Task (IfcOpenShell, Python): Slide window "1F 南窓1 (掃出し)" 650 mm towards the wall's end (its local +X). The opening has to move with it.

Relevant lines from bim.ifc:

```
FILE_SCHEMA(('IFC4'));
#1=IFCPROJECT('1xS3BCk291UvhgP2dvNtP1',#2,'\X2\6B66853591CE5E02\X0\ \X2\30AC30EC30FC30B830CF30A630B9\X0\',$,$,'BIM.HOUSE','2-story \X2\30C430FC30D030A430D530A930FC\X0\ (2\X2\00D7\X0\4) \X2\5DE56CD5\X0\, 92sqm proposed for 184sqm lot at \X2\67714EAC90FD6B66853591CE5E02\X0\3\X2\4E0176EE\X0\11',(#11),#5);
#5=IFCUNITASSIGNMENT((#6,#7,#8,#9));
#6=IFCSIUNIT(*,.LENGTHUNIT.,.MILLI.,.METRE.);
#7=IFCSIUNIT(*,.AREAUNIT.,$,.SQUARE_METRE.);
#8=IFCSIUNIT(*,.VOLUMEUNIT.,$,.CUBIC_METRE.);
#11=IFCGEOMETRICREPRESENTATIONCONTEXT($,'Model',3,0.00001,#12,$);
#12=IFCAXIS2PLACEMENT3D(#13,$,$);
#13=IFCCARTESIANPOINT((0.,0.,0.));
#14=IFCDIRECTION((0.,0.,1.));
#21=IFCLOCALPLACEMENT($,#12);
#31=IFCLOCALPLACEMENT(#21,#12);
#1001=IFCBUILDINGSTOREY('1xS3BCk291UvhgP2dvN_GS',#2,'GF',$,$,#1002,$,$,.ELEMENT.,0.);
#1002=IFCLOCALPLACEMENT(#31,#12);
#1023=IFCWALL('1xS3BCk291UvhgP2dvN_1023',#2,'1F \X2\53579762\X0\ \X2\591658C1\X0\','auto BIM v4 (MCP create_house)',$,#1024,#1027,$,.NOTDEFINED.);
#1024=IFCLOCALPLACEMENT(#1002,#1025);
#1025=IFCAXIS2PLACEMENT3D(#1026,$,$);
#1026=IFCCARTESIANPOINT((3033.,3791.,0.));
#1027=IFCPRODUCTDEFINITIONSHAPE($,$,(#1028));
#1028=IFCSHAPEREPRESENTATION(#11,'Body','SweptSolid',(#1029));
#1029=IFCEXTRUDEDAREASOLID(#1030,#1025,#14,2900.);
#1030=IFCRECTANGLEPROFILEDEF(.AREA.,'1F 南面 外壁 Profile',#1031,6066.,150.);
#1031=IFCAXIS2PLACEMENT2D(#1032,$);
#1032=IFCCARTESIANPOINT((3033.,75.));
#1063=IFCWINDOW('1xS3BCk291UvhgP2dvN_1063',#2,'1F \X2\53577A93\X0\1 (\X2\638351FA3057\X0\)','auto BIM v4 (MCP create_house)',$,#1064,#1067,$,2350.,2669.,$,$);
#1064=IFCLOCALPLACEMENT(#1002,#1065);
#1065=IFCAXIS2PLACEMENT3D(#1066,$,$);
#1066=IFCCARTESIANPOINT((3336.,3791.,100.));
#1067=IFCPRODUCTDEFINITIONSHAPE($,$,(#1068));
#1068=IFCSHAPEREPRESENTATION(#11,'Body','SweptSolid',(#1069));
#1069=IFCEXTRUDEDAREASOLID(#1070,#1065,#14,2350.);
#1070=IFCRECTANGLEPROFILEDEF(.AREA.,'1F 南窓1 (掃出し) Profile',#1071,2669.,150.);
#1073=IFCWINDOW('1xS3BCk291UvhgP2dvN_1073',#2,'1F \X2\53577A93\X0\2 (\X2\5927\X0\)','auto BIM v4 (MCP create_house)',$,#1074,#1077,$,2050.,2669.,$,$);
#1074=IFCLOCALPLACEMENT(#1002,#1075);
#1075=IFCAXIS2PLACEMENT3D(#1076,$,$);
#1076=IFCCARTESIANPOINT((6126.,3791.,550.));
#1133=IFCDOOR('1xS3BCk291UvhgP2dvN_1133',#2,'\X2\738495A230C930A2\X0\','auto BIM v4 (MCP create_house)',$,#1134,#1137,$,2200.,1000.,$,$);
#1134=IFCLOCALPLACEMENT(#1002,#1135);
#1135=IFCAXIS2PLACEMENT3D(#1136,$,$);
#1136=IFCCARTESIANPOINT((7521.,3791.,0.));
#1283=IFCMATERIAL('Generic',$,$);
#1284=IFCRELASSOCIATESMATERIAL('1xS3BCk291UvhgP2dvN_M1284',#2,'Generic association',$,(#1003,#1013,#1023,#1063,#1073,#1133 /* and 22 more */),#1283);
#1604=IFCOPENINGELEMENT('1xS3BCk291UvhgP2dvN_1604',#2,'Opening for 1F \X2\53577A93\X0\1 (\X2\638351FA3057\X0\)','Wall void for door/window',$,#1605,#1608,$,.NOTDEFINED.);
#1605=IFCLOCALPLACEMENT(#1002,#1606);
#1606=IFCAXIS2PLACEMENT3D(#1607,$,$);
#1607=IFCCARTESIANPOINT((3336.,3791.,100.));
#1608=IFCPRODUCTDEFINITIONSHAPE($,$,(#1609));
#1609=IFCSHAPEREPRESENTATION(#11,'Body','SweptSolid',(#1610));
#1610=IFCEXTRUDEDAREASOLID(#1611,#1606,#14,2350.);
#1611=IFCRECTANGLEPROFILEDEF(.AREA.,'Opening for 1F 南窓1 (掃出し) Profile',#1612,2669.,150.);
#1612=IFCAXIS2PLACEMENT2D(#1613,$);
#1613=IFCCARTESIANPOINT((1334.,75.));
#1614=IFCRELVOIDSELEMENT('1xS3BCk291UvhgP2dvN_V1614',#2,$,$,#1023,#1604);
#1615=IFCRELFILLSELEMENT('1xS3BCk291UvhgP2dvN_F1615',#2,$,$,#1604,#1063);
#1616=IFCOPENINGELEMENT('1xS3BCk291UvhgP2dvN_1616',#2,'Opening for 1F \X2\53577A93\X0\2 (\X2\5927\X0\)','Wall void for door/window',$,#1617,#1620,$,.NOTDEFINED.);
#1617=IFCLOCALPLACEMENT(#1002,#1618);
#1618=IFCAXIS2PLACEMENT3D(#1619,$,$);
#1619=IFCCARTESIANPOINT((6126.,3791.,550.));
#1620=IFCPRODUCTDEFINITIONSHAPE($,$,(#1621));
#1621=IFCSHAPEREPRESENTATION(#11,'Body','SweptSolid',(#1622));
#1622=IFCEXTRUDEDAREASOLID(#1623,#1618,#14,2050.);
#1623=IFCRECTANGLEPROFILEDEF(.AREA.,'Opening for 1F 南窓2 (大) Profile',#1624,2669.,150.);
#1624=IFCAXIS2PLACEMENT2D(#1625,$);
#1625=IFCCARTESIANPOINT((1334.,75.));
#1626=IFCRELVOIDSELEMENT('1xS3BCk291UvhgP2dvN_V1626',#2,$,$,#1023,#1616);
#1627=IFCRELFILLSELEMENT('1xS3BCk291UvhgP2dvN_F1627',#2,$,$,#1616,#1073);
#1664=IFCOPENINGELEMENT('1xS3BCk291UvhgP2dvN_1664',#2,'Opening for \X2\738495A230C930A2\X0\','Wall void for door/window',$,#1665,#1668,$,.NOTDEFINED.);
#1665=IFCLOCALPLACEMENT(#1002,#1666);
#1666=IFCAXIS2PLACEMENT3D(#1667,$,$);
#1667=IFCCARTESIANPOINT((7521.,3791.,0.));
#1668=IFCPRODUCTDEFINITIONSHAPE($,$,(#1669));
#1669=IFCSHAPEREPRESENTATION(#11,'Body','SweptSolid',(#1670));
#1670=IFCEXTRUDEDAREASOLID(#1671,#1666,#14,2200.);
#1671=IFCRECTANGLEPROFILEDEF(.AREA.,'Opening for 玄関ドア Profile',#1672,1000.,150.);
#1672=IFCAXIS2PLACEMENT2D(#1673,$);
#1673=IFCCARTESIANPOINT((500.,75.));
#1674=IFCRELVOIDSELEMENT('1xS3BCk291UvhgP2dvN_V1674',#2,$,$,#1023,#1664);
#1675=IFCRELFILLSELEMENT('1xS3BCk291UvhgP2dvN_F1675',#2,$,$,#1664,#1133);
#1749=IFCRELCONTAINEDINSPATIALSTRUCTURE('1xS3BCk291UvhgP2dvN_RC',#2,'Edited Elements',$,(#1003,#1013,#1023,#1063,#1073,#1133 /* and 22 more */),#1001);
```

```python
import ifcopenshell
import ifcopenshell.api.geometry
import ifcopenshell.util.placement
import ifcopenshell.util.unit

model = ifcopenshell.open("bim.ifc")
unit_scale = ifcopenshell.util.unit.calculate_unit_scale(model)

window = model.by_guid("1xS3BCk291UvhgP2dvN_1063")
opening = window.FillsVoids[0].RelatingOpeningElement
wall = opening.VoidsElements[0].RelatingBuildingElement

wall_matrix = ifcopenshell.util.placement.get_local_placement(wall.ObjectPlacement)
shift = wall_matrix[:3, 0] * 0.65 / unit_scale
before = ifcopenshell.util.placement.get_local_placement(window.ObjectPlacement)[:3, 3].copy()

# The window is not placed relative to its opening, so move both.
for product in (opening, window):
    matrix = ifcopenshell.util.placement.get_local_placement(product.ObjectPlacement)
    matrix[:3, 3] += shift
    ifcopenshell.api.geometry.edit_object_placement(model, product=product, matrix=matrix, is_si=False)

after = ifcopenshell.util.placement.get_local_placement(window.ObjectPlacement)[:3, 3]
print("window moved by", (after - before).round(3) + 0.0)

model.write("bim_rev.ifc")
```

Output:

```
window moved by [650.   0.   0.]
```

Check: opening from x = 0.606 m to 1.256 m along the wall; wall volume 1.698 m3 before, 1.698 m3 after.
